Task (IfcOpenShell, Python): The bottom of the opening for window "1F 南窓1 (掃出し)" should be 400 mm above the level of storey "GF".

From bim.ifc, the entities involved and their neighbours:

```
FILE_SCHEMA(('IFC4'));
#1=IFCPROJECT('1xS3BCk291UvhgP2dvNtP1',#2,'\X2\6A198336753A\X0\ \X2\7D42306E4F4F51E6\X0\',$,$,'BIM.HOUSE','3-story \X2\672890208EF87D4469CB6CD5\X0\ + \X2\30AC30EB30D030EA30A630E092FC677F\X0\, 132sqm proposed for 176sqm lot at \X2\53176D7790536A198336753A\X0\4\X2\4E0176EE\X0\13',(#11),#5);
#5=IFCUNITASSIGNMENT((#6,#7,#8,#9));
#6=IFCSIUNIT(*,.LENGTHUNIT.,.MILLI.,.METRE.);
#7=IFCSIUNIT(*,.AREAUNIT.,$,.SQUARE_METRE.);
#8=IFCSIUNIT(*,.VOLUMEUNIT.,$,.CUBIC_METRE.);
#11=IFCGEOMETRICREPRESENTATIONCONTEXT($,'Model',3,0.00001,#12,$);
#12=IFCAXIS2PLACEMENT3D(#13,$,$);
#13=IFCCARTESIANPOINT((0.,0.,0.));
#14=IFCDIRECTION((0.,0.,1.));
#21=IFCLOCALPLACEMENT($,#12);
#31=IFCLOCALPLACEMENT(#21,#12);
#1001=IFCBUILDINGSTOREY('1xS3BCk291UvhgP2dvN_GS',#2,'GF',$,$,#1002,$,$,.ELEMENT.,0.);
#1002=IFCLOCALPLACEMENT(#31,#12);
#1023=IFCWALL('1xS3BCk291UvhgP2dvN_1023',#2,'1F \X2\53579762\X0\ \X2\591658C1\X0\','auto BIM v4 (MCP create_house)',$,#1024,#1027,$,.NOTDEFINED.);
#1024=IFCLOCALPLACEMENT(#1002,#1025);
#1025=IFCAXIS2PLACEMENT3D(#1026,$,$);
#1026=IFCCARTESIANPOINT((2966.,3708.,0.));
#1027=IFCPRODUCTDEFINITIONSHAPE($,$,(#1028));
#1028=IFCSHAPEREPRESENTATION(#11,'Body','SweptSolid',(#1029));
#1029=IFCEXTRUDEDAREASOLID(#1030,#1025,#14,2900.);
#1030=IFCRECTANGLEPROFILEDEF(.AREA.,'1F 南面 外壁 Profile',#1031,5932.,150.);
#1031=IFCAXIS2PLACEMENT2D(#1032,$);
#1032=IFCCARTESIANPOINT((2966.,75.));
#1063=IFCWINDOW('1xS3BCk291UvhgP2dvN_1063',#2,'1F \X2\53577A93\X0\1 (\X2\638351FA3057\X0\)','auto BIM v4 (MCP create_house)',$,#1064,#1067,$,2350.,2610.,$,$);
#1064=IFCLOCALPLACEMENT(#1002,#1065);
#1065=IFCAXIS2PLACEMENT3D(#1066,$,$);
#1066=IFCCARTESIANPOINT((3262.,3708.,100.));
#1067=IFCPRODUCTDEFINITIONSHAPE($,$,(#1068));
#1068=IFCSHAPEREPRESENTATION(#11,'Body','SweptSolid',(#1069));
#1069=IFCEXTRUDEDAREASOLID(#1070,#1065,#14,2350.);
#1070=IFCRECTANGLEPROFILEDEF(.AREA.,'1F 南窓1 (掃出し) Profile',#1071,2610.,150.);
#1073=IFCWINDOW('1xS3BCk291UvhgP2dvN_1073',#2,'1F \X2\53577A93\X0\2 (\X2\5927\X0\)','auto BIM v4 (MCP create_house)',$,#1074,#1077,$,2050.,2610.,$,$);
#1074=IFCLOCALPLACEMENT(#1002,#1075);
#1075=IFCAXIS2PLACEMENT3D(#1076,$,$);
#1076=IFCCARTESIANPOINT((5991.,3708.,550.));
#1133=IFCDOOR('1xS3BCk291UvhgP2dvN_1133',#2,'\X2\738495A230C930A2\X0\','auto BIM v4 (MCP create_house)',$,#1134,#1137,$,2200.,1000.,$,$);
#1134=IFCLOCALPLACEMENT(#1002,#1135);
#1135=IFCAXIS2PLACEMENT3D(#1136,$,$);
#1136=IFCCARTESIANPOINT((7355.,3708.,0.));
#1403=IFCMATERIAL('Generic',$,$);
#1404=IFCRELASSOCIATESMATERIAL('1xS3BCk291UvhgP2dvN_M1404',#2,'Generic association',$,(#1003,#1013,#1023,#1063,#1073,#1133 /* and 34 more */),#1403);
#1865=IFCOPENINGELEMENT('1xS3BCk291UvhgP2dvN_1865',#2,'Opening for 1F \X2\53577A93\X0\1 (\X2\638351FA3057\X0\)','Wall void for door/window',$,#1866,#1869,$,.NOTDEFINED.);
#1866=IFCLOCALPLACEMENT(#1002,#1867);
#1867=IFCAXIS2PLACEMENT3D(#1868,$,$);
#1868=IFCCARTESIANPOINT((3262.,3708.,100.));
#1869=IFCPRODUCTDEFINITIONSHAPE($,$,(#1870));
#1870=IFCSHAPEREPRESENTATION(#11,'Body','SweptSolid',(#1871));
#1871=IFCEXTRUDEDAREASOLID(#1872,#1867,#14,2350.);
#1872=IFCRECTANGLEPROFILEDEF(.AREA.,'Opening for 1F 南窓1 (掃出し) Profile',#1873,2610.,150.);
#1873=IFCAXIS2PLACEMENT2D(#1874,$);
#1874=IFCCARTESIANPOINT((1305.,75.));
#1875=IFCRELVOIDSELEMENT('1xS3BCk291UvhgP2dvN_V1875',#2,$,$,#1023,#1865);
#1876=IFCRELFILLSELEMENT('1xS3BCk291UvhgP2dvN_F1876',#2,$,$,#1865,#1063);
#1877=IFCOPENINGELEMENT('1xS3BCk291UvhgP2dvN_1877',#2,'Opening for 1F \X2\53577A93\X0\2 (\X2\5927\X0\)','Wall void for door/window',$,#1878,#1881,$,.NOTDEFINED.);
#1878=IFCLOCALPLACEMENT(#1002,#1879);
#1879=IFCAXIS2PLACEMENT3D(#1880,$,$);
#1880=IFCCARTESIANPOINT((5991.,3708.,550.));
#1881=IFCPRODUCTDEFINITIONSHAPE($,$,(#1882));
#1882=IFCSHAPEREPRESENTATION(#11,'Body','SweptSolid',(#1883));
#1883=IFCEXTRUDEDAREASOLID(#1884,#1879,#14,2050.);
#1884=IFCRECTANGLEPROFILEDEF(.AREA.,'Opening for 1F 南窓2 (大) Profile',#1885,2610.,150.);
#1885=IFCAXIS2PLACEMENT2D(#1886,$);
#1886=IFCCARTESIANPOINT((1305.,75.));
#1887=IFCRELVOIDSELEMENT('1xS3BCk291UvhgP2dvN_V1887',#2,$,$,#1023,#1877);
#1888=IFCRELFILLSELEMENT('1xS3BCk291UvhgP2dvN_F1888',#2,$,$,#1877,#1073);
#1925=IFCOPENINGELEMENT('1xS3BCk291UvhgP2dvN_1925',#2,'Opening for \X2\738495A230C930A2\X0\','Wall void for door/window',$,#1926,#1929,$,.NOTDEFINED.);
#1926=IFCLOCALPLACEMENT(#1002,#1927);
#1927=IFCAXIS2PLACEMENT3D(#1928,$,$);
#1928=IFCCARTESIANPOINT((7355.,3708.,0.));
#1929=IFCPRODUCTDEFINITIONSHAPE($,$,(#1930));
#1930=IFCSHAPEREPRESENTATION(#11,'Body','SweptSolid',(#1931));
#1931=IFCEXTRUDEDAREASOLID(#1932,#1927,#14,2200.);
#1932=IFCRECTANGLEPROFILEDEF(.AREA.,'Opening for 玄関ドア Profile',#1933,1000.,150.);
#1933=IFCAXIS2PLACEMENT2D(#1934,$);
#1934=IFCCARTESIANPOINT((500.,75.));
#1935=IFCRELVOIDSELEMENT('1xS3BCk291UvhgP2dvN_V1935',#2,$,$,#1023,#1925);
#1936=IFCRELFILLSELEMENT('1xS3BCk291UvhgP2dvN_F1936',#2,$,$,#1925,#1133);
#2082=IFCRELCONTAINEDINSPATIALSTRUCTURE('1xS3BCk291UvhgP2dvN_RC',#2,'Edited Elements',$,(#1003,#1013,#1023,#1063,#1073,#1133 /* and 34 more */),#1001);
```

```python
import numpy as np
import ifcopenshell
import ifcopenshell.api.geometry
import ifcopenshell.geom
import ifcopenshell.util.element
import ifcopenshell.util.placement
import ifcopenshell.util.shape
import ifcopenshell.util.unit

model = ifcopenshell.open("bim.ifc")
unit_scale = ifcopenshell.util.unit.calculate_unit_scale(model)

window = model.by_guid("1xS3BCk291UvhgP2dvN_1063")
opening = window.FillsVoids[0].RelatingOpeningElement
storey = ifcopenshell.util.element.get_container(window, ifc_class="IfcBuildingStorey")
level = ifcopenshell.util.placement.get_local_placement(storey.ObjectPlacement)[2, 3]

# The opening's origin need not be at the sill, so measure its lowest point.
shape = ifcopenshell.geom.create_shape(ifcopenshell.geom.settings(), opening)
bottom = ifcopenshell.util.shape.get_shape_bottom_elevation(shape, shape.geometry) / unit_scale
dz = level + 400.0 - bottom

shift = np.array([0.0, 0.0, dz])
# The window is not placed relative to its opening, so move both.
for product in (opening, window):
    matrix = ifcopenshell.util.placement.get_local_placement(product.ObjectPlacement)
    matrix[:3, 3] += shift
    ifcopenshell.api.geometry.edit_object_placement(model, product=product, matrix=matrix, is_si=False)

print(f"moved by {dz * unit_scale:+.3f} m")

model.write("bim_updated.ifc")
```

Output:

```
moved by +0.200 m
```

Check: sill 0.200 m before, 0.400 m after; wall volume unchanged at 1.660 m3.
